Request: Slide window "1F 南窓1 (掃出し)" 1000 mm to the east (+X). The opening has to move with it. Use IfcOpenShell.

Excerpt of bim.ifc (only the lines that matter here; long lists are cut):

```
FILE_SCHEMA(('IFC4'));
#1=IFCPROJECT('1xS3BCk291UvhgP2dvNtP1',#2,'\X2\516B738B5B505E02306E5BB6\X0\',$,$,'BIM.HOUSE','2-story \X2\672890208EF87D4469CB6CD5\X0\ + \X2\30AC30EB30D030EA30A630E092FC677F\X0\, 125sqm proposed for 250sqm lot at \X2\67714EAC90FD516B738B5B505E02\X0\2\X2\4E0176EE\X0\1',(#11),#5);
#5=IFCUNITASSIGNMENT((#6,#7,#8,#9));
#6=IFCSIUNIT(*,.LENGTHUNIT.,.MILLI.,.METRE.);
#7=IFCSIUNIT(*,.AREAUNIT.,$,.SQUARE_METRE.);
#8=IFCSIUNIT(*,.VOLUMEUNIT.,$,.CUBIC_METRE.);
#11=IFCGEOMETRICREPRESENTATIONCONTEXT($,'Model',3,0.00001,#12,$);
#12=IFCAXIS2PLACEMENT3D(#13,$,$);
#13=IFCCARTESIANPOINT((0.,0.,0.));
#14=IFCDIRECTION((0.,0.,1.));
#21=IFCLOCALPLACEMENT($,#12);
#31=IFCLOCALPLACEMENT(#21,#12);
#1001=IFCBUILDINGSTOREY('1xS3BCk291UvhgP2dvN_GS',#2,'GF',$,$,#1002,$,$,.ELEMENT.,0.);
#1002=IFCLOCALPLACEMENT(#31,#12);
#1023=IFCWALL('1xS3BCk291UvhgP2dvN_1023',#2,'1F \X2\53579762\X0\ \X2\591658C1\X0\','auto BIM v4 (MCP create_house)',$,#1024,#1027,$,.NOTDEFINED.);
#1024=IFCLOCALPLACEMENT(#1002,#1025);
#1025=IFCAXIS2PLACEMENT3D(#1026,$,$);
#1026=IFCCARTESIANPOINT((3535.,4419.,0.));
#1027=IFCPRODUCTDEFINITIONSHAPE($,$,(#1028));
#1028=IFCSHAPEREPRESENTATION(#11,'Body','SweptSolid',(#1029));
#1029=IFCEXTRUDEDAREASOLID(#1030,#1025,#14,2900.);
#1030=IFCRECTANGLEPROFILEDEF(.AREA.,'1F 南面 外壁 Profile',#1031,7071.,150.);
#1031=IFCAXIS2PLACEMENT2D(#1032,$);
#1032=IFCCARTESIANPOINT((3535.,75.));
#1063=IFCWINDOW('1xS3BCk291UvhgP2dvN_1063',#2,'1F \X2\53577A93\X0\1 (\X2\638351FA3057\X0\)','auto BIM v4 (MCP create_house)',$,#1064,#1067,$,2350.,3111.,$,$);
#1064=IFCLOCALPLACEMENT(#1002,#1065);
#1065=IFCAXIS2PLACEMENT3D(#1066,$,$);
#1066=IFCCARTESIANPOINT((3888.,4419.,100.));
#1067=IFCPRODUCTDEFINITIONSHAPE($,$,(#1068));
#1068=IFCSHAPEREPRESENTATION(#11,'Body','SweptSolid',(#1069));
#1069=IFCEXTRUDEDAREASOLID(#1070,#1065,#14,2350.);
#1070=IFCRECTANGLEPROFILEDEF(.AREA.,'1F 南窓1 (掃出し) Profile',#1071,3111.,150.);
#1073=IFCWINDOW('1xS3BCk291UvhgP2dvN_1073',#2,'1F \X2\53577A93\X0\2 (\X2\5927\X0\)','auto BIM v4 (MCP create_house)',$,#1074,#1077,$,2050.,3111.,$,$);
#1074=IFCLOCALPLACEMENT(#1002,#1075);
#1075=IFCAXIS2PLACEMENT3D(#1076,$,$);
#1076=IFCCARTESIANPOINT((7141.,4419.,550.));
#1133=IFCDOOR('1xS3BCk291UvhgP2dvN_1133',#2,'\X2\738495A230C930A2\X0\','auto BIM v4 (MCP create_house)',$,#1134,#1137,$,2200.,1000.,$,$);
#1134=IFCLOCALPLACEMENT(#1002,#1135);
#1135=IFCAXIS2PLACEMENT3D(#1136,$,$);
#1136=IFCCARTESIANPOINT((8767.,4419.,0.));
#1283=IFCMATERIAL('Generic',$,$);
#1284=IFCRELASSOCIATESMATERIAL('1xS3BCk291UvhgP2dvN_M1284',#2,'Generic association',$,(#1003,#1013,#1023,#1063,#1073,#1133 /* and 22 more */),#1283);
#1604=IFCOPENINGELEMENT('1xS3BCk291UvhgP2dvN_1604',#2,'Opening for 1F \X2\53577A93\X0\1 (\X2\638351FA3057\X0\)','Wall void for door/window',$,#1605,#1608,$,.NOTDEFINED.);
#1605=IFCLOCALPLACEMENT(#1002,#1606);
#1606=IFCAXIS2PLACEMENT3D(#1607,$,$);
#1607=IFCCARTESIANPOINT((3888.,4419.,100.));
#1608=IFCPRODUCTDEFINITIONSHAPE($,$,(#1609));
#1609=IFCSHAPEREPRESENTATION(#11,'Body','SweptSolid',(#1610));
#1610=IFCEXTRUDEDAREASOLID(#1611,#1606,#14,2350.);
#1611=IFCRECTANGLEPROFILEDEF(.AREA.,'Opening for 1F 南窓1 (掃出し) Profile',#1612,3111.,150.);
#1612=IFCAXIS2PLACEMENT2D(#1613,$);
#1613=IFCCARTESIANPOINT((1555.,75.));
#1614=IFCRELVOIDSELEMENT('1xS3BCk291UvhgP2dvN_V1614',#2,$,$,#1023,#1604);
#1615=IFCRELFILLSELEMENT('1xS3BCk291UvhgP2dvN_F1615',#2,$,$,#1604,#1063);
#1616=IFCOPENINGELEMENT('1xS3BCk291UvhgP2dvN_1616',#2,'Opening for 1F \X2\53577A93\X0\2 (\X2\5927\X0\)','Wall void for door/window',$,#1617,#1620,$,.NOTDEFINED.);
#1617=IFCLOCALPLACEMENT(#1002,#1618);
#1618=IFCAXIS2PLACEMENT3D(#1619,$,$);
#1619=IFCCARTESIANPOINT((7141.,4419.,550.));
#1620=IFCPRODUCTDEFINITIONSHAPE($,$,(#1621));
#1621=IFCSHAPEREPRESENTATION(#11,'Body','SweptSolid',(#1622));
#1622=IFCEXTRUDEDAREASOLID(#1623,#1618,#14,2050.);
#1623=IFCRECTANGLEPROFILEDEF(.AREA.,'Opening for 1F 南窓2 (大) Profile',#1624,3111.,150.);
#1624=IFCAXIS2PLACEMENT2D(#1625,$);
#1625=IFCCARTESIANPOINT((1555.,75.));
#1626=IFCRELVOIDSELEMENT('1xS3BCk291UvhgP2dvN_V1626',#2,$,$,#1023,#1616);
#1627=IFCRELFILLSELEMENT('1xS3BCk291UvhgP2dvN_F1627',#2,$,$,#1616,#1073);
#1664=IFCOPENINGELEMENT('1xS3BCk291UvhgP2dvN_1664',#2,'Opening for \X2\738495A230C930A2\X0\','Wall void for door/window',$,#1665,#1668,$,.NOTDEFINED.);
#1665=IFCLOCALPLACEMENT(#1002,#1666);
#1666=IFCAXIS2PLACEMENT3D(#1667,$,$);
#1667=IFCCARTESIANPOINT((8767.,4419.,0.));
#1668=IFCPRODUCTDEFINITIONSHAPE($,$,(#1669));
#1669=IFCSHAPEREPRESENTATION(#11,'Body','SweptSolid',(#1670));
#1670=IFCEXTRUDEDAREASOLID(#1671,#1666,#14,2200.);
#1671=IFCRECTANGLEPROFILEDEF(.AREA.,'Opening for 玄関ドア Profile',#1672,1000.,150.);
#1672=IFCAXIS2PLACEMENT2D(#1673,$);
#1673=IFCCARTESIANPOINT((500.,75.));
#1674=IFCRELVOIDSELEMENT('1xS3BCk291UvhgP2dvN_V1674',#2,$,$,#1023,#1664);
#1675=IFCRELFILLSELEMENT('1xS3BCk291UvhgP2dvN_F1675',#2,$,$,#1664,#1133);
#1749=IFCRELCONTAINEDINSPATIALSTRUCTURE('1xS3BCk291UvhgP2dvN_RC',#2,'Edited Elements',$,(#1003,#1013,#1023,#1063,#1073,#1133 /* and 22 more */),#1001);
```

```python
import ifcopenshell
import ifcopenshell.api.geometry
import ifcopenshell.util.placement
import ifcopenshell.util.unit

model = ifcopenshell.open("bim.ifc")
unit_scale = ifcopenshell.util.unit.calculate_unit_scale(model)

window = model.by_guid("1xS3BCk291UvhgP2dvN_1063")
opening = window.FillsVoids[0].RelatingOpeningElement
wall = opening.VoidsElements[0].RelatingBuildingElement

wall_matrix = ifcopenshell.util.placement.get_local_placement(wall.ObjectPlacement)
shift = wall_matrix[:3, 0] * 1 / unit_scale
before = ifcopenshell.util.placement.get_local_placement(window.ObjectPlacement)[:3, 3].copy()

# The window is not placed relative to its opening, so move both.
for product in (opening, window):
    matrix = ifcopenshell.util.placement.get_local_placement(product.ObjectPlacement)
    matrix[:3, 3] += shift
    ifcopenshell.api.geometry.edit_object_placement(model, product=product, matrix=matrix, is_si=False)

after = ifcopenshell.util.placement.get_local_placement(window.ObjectPlacement)[:3, 3]
print("window moved by", (after - before).round(3) + 0.0)

model.write("bim_edited.ifc")
```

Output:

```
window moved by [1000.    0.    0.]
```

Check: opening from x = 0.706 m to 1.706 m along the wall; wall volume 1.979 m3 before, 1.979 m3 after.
